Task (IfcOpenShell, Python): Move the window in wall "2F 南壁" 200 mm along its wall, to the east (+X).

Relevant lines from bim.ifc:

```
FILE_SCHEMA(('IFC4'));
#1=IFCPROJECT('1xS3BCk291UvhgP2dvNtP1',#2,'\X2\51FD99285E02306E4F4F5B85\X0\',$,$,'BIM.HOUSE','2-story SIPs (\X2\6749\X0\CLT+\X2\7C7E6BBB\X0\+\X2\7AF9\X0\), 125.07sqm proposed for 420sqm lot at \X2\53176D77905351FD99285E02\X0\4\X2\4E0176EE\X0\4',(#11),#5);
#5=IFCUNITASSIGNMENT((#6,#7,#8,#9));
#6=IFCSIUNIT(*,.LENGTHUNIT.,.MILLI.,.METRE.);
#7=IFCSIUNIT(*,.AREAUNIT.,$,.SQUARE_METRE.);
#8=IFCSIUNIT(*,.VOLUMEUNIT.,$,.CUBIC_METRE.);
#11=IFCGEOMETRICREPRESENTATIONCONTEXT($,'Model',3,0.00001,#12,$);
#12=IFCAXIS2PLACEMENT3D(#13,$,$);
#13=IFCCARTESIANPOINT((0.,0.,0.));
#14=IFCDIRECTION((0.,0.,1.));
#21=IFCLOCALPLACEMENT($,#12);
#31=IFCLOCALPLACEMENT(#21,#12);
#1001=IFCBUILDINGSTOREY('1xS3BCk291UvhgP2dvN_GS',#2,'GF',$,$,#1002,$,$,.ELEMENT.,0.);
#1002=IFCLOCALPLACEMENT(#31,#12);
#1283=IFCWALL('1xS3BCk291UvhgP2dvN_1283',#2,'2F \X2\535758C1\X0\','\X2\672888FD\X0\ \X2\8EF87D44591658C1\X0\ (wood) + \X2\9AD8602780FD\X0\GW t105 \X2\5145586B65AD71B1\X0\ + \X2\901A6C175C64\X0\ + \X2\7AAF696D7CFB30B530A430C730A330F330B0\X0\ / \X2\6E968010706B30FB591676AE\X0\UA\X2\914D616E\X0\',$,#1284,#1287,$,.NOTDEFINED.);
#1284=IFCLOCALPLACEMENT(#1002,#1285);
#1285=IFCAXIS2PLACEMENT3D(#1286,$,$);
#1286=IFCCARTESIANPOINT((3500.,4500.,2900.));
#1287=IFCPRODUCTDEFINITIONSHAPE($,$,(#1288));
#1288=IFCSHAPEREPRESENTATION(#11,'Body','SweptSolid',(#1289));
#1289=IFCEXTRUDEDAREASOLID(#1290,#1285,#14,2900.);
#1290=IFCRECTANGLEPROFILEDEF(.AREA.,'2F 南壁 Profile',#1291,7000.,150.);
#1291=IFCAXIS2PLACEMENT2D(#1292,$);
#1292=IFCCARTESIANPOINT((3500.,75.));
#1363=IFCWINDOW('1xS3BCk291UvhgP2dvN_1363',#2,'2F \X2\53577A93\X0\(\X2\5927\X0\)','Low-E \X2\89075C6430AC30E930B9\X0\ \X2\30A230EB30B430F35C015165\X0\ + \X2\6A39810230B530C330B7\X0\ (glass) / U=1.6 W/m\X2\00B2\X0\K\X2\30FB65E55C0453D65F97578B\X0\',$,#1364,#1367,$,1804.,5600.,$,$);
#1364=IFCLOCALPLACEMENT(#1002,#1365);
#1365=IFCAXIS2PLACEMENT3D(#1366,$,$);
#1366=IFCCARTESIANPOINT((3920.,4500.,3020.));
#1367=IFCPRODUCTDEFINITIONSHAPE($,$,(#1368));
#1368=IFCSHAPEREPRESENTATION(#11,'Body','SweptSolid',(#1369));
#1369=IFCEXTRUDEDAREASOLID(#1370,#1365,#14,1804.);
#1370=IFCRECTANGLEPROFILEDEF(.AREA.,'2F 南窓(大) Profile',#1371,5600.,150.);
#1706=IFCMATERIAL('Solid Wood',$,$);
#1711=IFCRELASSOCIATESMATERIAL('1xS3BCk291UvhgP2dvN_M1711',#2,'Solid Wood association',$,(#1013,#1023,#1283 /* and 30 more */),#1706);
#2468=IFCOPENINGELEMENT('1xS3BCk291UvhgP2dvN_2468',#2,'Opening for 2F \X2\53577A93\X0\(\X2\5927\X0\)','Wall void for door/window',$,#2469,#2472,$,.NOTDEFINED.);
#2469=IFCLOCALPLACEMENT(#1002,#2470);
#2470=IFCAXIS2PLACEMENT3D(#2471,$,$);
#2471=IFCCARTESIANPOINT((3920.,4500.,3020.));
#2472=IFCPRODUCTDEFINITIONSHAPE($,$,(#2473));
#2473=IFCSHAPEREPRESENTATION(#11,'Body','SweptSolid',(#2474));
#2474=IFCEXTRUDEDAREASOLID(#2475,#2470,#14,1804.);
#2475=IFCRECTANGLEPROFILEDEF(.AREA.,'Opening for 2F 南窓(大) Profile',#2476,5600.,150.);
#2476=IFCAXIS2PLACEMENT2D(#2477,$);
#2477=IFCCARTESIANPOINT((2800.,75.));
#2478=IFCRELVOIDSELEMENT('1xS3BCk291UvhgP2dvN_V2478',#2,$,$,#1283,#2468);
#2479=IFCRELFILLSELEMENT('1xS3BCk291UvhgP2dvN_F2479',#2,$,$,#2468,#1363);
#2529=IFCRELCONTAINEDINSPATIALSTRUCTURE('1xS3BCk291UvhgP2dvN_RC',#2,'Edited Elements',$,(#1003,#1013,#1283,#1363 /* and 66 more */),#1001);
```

```python
import ifcopenshell
import ifcopenshell.api.geometry
import ifcopenshell.util.placement
import ifcopenshell.util.unit

model = ifcopenshell.open("bim.ifc")
unit_scale = ifcopenshell.util.unit.calculate_unit_scale(model)

window = model.by_guid("1xS3BCk291UvhgP2dvN_1363")
opening = window.FillsVoids[0].RelatingOpeningElement
wall = opening.VoidsElements[0].RelatingBuildingElement

wall_matrix = ifcopenshell.util.placement.get_local_placement(wall.ObjectPlacement)
shift = wall_matrix[:3, 0] * 0.2 / unit_scale
before = ifcopenshell.util.placement.get_local_placement(window.ObjectPlacement)[:3, 3].copy()

# The window is not placed relative to its opening, so move both.
for product in (opening, window):
    matrix = ifcopenshell.util.placement.get_local_placement(product.ObjectPlacement)
    matrix[:3, 3] += shift
    ifcopenshell.api.geometry.edit_object_placement(model, product=product, matrix=matrix, is_si=False)

after = ifcopenshell.util.placement.get_local_placement(window.ObjectPlacement)[:3, 3]
print("window moved by", (after - before).round(3) + 0.0)

model.write("bim_v2.ifc")
```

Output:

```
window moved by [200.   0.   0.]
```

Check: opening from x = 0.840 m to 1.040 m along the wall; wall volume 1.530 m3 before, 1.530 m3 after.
